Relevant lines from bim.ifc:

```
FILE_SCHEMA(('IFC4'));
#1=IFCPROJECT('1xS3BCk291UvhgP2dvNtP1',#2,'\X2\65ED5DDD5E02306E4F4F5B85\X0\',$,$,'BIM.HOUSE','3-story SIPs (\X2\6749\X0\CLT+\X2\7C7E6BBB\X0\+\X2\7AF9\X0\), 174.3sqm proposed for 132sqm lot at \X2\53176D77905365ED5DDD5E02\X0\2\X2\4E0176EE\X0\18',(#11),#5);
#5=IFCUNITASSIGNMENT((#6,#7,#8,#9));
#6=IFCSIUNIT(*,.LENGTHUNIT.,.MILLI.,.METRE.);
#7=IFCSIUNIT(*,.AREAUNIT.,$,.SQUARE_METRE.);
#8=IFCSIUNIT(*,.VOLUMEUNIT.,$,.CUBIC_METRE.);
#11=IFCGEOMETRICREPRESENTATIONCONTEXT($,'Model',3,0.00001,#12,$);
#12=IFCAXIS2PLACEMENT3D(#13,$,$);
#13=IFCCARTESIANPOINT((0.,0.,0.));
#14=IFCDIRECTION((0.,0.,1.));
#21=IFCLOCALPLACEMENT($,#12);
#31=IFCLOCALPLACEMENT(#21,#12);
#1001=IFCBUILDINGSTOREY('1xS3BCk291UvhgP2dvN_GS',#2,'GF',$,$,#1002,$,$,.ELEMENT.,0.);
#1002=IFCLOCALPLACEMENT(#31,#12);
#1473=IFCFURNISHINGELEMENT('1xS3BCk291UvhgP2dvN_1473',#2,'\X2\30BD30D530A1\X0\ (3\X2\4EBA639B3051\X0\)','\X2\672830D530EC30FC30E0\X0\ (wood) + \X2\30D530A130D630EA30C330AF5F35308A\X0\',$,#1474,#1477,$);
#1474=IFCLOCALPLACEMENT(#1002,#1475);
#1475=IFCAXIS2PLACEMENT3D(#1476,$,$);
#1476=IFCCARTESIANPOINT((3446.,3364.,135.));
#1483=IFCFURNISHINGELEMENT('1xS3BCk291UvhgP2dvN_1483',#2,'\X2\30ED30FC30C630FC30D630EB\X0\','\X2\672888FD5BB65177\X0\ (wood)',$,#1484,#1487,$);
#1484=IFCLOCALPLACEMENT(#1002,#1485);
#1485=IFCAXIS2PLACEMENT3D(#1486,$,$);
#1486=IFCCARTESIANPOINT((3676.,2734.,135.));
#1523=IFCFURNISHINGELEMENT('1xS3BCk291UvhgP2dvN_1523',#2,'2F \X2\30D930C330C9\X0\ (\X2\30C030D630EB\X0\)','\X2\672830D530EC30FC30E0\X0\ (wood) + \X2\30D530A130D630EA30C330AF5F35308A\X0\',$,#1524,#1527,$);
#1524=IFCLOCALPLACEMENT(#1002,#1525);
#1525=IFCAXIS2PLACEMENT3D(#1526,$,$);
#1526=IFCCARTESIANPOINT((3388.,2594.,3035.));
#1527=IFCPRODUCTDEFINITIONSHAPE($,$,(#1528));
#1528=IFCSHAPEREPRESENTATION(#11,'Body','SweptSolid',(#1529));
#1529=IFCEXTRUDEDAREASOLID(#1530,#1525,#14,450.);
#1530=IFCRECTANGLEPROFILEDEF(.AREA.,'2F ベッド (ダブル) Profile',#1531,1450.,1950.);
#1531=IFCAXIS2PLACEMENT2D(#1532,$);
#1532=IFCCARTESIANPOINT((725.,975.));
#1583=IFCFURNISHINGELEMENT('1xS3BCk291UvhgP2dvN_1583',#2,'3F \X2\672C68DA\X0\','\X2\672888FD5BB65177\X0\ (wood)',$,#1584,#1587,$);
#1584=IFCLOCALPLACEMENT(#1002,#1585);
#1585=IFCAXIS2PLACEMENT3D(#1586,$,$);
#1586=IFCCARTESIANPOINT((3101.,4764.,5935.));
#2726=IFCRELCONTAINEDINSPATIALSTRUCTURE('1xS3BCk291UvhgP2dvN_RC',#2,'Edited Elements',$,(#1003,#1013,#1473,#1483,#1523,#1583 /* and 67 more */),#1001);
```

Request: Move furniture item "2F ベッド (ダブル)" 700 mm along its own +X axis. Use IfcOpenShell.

```python
import ifcopenshell
import ifcopenshell.api.geometry
import ifcopenshell.util.placement
import ifcopenshell.util.unit

model = ifcopenshell.open("bim.ifc")
unit_scale = ifcopenshell.util.unit.calculate_unit_scale(model)

item = model.by_guid("1xS3BCk291UvhgP2dvN_1523")
matrix = ifcopenshell.util.placement.get_local_placement(item.ObjectPlacement)
matrix[:3, 3] += matrix[:3, 0] * 0.7 / unit_scale
ifcopenshell.api.geometry.edit_object_placement(model, product=item, matrix=matrix, is_si=False)

print(ifcopenshell.util.placement.get_local_placement(item.ObjectPlacement).round(3) + 0.0)

model.write("bim_v2.ifc")
```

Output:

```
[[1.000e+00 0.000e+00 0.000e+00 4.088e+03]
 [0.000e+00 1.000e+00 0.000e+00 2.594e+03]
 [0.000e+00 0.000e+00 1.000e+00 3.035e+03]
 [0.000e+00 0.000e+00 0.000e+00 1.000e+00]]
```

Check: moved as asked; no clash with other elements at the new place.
